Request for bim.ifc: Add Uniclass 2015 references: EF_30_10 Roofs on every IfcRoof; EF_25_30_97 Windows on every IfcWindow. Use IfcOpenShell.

First a look at what the model holds.

```python
import ifcopenshell

model = ifcopenshell.open("bim.ifc")
print(model.schema)
print("classifications:", [c.Name for c in model.by_type("IfcClassification")])
for ifc_class in ("IfcDoor", "IfcRoof", "IfcStair", "IfcWall", "IfcWindow"):
    print(ifc_class, len(model.by_type(ifc_class)))
```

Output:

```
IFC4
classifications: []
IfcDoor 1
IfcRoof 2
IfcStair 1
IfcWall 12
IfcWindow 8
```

```python
import ifcopenshell
import ifcopenshell.api.classification

model = ifcopenshell.open("bim.ifc")

system = ifcopenshell.api.classification.add_classification(model, classification="Uniclass 2015")

codes = {
    "IfcRoof": ("EF_30_10", "Roofs"),
    "IfcWindow": ("EF_25_30_97", "Windows"),
}
for ifc_class, (code, name) in codes.items():
    products = model.by_type(ifc_class)
    ifcopenshell.api.classification.add_reference(
        model, products=products, classification=system, identification=code, name=name
    )
    print(code, len(products))

model.write("bim_updated.ifc")
```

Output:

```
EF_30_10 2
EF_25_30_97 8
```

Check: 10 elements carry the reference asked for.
